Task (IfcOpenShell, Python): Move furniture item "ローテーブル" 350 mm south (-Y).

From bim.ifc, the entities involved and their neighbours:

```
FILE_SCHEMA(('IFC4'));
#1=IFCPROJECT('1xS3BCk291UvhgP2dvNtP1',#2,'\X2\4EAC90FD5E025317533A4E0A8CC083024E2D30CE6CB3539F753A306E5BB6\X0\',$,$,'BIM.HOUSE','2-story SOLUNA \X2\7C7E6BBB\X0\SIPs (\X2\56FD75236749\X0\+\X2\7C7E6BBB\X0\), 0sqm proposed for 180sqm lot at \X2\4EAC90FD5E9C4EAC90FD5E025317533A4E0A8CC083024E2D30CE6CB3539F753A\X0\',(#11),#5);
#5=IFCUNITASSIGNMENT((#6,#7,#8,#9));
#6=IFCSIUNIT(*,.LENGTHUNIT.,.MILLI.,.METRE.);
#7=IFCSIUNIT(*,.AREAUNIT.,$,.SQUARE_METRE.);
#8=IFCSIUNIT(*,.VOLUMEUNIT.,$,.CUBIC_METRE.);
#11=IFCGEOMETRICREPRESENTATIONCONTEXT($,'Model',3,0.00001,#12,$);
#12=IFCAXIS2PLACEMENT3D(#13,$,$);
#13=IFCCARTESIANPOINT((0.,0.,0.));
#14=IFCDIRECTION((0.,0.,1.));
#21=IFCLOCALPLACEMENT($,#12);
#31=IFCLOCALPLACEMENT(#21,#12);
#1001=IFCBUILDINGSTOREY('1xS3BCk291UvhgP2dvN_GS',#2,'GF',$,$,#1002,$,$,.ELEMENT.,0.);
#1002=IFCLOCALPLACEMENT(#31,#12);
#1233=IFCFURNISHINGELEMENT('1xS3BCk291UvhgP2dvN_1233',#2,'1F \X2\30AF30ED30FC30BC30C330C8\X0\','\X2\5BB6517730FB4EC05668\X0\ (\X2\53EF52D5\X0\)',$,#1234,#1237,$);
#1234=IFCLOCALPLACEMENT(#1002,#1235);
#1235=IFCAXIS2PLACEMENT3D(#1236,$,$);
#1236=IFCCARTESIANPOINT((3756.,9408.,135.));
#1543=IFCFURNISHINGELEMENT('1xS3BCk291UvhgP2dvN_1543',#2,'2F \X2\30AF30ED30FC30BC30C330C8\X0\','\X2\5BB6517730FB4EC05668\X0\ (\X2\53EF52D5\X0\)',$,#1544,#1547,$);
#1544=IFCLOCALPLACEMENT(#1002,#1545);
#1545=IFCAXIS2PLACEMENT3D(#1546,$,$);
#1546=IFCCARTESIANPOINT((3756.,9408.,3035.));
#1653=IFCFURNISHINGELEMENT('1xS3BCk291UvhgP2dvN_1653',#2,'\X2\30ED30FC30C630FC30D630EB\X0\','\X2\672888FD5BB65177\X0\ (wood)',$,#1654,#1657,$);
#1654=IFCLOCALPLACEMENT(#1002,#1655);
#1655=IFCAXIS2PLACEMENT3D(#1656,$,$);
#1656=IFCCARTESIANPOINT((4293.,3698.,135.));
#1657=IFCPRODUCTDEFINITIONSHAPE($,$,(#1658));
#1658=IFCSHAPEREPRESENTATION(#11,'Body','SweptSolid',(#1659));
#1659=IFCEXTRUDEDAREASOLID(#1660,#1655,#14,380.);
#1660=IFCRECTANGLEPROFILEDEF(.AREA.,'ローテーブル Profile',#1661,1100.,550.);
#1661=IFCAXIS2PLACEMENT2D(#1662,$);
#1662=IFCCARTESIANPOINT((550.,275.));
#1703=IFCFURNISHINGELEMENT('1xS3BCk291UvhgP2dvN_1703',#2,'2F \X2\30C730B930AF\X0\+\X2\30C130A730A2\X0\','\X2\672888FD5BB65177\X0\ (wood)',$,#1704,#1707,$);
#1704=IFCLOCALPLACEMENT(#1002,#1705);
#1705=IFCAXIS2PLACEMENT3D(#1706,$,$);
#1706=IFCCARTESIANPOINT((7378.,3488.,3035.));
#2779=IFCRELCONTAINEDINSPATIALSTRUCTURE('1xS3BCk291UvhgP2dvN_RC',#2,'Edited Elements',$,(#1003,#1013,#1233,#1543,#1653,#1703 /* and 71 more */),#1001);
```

```python
import ifcopenshell
import ifcopenshell.api.geometry
import ifcopenshell.util.placement
import ifcopenshell.util.unit

model = ifcopenshell.open("bim.ifc")
unit_scale = ifcopenshell.util.unit.calculate_unit_scale(model)

item = model.by_id(1653)
matrix = ifcopenshell.util.placement.get_local_placement(item.ObjectPlacement)
matrix[1, 3] -= 0.35 / unit_scale
ifcopenshell.api.geometry.edit_object_placement(model, product=item, matrix=matrix, is_si=False)

print(ifcopenshell.util.placement.get_local_placement(item.ObjectPlacement).round(3) + 0.0)

model.write("bim-out.ifc")
```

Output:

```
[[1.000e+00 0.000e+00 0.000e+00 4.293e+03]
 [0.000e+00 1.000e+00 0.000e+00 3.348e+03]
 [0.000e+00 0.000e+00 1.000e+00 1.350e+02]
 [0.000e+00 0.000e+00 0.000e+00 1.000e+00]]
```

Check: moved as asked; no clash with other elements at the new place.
